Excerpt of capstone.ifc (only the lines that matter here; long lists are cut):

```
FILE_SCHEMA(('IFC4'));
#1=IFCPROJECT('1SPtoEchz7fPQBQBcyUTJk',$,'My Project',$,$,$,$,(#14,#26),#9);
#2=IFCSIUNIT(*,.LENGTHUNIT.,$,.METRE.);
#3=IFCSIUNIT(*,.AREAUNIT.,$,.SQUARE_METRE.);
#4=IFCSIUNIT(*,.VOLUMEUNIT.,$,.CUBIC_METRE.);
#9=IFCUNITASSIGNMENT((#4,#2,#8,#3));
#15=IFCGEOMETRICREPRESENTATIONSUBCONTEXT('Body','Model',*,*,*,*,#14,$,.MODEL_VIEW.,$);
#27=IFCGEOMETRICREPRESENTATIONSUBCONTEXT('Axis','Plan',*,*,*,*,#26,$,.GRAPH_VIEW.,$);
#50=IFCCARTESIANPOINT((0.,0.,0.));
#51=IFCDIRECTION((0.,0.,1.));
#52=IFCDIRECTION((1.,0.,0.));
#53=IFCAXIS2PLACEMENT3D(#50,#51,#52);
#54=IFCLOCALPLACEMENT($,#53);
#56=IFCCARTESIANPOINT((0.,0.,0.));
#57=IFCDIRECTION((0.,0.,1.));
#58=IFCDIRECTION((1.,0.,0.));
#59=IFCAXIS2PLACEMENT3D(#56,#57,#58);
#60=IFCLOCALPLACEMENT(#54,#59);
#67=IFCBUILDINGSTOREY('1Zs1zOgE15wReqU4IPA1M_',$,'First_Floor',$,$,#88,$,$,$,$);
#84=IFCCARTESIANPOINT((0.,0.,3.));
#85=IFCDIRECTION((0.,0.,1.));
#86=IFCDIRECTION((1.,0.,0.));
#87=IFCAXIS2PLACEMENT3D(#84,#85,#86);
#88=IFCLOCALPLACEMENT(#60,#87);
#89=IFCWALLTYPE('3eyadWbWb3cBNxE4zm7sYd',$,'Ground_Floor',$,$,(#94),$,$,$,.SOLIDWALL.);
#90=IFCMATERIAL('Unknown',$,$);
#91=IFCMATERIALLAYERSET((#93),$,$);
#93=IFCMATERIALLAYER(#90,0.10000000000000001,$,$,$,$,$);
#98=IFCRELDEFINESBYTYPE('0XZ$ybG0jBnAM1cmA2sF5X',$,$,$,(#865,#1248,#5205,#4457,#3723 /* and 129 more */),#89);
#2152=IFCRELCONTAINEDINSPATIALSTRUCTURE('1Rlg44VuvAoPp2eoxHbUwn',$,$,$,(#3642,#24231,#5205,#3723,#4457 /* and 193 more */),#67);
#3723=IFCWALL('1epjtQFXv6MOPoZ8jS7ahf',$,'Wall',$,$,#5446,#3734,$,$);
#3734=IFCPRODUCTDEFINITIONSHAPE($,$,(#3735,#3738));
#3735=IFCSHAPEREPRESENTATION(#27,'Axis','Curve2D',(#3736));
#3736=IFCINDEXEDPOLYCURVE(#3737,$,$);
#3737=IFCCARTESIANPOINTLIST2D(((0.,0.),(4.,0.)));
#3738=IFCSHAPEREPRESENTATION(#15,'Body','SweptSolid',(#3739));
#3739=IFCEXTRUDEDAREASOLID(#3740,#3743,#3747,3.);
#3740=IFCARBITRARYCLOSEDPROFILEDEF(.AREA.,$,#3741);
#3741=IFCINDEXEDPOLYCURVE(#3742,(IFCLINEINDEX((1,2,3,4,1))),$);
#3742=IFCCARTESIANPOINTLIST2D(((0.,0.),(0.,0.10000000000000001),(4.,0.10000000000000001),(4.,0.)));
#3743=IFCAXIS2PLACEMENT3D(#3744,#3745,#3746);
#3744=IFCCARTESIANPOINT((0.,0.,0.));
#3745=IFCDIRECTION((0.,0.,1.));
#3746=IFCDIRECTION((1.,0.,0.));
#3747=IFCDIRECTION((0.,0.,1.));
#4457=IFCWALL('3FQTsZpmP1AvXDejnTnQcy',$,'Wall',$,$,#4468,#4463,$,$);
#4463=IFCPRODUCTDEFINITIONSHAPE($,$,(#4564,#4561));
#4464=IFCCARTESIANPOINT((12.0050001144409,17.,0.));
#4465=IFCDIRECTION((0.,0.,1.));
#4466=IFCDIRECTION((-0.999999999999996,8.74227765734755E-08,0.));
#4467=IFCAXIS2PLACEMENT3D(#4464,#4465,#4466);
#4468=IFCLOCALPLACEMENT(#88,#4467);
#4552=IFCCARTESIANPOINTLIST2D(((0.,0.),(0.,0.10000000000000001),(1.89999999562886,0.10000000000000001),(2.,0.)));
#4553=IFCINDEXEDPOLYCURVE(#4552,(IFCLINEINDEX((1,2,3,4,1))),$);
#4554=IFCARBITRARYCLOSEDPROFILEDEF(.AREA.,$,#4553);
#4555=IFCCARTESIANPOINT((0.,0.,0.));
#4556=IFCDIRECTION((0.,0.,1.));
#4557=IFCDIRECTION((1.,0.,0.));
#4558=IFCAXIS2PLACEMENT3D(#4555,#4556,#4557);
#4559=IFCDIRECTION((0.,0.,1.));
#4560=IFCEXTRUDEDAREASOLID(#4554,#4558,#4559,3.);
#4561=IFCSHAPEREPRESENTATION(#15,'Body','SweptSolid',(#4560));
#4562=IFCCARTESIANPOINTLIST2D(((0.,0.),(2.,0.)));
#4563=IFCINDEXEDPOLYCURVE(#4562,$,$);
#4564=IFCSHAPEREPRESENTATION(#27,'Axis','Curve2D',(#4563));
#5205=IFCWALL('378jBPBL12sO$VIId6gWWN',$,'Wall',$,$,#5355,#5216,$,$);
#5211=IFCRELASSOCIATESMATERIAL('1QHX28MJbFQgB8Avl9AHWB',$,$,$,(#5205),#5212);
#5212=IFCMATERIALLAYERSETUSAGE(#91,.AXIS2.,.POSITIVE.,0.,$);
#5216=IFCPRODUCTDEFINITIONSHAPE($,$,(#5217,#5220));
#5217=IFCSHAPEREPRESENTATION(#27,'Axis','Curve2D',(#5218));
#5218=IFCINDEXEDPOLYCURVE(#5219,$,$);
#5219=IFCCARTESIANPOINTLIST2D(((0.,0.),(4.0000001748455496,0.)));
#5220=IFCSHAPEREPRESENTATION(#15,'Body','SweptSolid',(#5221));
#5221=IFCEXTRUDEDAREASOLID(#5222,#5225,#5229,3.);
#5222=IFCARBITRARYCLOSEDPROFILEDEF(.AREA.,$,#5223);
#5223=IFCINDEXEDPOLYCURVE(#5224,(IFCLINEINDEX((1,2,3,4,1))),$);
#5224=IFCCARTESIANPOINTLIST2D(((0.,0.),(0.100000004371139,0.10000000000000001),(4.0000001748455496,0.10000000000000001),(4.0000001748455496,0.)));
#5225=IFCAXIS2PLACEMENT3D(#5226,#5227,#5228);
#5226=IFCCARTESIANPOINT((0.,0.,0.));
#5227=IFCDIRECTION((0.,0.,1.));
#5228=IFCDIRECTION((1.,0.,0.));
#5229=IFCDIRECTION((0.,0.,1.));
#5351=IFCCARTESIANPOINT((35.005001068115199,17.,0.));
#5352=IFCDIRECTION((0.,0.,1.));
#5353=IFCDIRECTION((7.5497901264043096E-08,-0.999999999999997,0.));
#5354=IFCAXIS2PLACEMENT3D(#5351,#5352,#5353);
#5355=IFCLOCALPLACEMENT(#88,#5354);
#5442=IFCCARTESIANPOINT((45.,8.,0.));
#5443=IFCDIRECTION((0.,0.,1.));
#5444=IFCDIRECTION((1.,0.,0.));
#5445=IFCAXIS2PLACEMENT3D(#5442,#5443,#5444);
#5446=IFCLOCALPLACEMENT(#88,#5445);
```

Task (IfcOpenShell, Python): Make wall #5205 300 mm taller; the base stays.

```python
import ifcopenshell
import ifcopenshell.geom
import ifcopenshell.util.representation
import ifcopenshell.util.shape
import ifcopenshell.util.unit

model = ifcopenshell.open("capstone.ifc")
unit_scale = ifcopenshell.util.unit.calculate_unit_scale(model)
settings = ifcopenshell.geom.settings()


def volume(element):
    """Net volume in cubic metres, openings subtracted."""
    shape = ifcopenshell.geom.create_shape(settings, element)
    return ifcopenshell.util.shape.get_volume(shape.geometry)


wall = model.by_id(5205)
before = volume(wall)

body = ifcopenshell.util.representation.get_representation(wall, "Model", "Body")
solid = body.Items[0]
old_height = solid.Depth
solid.Depth += 0.3 / unit_scale
after = volume(wall)

print(f"height {old_height:g} -> {solid.Depth:g}, volume {before:.3f} -> {after:.3f} m3")

model.write("capstone_edited.ifc")
```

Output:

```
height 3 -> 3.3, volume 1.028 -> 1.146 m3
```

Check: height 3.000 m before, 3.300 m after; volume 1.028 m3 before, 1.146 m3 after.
